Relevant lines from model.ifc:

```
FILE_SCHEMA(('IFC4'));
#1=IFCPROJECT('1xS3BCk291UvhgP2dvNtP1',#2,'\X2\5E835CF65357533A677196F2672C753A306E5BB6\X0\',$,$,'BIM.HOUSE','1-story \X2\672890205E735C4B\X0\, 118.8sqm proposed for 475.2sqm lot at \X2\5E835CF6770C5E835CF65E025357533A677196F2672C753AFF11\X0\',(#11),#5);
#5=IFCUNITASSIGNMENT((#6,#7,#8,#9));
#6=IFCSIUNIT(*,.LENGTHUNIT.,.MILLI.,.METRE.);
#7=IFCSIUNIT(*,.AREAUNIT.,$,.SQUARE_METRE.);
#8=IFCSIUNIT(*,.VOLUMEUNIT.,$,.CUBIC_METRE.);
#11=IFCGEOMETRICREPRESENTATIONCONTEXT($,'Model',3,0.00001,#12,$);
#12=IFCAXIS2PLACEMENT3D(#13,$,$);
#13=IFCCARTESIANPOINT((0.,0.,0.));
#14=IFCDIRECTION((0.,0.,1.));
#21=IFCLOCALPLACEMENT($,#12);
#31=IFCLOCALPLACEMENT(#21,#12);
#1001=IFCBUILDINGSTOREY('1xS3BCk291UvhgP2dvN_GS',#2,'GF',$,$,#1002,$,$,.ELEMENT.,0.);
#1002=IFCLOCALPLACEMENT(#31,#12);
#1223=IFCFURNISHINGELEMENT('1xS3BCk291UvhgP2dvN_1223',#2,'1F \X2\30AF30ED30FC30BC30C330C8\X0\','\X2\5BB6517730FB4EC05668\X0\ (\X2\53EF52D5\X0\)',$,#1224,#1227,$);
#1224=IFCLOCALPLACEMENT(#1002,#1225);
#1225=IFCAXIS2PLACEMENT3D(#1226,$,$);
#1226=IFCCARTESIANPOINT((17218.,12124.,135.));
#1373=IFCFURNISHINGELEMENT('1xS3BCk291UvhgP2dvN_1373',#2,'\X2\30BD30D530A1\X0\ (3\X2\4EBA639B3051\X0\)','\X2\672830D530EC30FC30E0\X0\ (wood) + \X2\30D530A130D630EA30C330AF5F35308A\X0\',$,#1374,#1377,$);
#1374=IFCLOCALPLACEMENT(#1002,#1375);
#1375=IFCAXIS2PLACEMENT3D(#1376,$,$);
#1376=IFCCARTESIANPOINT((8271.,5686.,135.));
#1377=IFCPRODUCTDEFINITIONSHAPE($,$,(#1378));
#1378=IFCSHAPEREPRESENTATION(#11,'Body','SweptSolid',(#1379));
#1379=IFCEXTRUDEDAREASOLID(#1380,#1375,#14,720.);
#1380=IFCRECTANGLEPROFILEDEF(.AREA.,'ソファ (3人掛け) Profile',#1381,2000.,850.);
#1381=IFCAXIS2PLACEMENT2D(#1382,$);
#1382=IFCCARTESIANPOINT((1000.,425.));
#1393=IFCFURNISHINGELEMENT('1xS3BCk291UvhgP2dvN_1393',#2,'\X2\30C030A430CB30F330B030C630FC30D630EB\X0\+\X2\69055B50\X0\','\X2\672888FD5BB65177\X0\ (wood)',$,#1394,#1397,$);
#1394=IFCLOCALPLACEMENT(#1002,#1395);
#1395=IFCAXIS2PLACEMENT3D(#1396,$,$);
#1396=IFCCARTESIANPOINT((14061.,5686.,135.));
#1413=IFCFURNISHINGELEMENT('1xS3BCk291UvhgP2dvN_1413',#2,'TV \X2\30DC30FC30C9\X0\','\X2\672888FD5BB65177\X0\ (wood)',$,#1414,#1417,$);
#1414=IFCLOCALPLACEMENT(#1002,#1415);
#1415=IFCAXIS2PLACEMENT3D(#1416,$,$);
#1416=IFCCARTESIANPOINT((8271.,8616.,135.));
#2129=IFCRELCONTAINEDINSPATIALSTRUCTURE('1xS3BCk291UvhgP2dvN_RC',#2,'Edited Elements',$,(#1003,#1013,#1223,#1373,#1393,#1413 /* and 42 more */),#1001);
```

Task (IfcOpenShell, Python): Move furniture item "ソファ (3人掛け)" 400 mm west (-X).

```python
import ifcopenshell
import ifcopenshell.api.geometry
import ifcopenshell.util.placement
import ifcopenshell.util.unit

model = ifcopenshell.open("model.ifc")
unit_scale = ifcopenshell.util.unit.calculate_unit_scale(model)

item = model.by_id(1373)
matrix = ifcopenshell.util.placement.get_local_placement(item.ObjectPlacement)
matrix[0, 3] -= 0.4 / unit_scale
ifcopenshell.api.geometry.edit_object_placement(model, product=item, matrix=matrix, is_si=False)

print(ifcopenshell.util.placement.get_local_placement(item.ObjectPlacement).round(3) + 0.0)

model.write("model_rev.ifc")
```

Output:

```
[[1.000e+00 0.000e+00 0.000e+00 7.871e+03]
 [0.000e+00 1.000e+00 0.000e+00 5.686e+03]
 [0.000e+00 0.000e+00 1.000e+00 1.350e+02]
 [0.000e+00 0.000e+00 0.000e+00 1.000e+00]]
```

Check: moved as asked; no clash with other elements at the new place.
